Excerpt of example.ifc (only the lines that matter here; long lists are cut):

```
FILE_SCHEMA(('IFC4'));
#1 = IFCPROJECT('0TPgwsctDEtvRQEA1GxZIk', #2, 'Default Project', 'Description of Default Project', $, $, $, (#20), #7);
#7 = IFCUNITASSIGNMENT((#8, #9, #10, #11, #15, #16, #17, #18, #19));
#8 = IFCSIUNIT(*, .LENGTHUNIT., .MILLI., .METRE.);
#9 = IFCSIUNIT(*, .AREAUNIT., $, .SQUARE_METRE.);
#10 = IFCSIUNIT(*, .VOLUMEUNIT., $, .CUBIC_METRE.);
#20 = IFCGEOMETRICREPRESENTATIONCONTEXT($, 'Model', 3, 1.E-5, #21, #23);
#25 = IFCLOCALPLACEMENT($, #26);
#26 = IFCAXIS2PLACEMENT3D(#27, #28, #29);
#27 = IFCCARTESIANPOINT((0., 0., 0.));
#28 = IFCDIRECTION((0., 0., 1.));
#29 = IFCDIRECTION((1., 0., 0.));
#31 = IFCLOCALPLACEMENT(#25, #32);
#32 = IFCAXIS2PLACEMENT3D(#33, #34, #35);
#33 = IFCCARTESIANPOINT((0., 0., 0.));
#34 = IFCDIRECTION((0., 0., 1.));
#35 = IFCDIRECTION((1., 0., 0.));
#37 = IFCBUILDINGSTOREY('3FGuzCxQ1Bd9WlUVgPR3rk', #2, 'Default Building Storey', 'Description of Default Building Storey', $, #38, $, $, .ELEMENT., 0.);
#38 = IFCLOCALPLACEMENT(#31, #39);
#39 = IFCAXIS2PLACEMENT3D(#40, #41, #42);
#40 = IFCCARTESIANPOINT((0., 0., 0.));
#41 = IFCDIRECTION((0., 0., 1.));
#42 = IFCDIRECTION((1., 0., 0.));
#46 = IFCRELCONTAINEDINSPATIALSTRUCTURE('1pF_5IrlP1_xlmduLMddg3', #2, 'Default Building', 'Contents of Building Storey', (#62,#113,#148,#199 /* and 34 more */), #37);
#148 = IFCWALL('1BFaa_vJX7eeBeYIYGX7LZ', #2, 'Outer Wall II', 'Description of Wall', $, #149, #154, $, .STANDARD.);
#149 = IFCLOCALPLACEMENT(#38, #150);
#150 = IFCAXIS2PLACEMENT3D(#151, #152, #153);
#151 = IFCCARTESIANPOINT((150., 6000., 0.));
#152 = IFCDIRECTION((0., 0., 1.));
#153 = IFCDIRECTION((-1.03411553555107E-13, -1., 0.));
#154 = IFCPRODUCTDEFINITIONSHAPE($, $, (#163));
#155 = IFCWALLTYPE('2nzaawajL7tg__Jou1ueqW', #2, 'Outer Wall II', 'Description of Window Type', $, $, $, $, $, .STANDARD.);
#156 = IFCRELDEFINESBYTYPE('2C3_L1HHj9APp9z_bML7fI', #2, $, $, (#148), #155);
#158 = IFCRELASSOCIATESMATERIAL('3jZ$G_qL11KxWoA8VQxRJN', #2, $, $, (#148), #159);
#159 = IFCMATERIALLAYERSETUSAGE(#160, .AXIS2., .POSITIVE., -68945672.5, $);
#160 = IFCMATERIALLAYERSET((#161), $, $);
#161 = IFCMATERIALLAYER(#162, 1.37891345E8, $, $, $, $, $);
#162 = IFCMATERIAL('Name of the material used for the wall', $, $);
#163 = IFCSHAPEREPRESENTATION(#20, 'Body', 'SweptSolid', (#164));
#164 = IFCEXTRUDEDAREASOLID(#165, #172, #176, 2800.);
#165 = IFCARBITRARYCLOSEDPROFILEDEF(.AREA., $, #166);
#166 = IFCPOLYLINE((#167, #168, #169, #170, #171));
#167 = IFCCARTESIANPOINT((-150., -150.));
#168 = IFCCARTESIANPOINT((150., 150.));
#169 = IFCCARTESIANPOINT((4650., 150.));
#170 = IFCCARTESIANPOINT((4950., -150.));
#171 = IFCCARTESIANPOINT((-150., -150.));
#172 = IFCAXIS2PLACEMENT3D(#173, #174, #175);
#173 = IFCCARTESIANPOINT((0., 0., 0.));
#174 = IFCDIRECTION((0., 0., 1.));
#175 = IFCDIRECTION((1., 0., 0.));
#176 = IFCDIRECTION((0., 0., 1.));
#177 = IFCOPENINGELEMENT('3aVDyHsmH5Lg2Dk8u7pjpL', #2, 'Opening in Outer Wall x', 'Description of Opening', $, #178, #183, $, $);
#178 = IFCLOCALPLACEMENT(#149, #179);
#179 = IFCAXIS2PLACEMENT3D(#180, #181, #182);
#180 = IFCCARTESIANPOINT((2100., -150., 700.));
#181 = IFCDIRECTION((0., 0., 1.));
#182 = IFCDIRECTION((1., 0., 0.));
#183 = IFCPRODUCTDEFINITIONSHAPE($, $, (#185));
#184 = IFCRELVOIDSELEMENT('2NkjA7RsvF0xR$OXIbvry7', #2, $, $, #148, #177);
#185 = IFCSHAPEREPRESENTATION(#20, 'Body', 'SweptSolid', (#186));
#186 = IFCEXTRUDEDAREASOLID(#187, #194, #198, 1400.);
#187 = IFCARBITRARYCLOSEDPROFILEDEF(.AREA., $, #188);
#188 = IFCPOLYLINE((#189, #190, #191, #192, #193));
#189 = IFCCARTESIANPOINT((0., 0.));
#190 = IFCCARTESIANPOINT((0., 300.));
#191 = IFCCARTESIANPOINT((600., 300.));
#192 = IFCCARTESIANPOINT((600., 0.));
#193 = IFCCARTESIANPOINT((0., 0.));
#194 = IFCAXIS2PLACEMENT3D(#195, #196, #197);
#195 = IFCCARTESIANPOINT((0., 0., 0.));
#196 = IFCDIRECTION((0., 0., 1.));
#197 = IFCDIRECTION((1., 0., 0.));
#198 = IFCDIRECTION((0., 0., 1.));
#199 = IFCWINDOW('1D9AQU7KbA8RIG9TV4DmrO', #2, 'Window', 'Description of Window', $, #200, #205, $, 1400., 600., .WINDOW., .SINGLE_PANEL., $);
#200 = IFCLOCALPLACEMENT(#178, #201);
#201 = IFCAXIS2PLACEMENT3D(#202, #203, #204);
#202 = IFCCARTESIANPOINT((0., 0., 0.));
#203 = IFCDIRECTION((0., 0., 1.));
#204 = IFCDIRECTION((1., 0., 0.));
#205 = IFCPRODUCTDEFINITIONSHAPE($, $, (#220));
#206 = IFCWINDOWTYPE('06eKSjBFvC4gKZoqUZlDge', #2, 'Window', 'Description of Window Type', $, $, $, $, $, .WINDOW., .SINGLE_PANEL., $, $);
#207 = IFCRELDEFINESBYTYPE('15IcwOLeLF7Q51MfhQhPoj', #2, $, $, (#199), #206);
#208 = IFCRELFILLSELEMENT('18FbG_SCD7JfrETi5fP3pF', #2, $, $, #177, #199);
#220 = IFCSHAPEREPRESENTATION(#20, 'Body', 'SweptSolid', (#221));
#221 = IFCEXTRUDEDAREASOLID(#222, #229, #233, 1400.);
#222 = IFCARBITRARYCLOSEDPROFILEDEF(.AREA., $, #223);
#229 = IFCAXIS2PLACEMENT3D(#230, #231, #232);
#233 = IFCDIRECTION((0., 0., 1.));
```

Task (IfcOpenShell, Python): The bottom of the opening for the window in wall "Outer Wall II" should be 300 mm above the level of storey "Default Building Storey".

```python
import numpy as np
import ifcopenshell
import ifcopenshell.api.geometry
import ifcopenshell.geom
import ifcopenshell.util.element
import ifcopenshell.util.placement
import ifcopenshell.util.shape
import ifcopenshell.util.unit

model = ifcopenshell.open("example.ifc")
unit_scale = ifcopenshell.util.unit.calculate_unit_scale(model)

window = model.by_guid("1D9AQU7KbA8RIG9TV4DmrO")
opening = window.FillsVoids[0].RelatingOpeningElement
storey = ifcopenshell.util.element.get_container(window, ifc_class="IfcBuildingStorey")
level = ifcopenshell.util.placement.get_local_placement(storey.ObjectPlacement)[2, 3]

# The opening's origin need not be at the sill, so measure its lowest point.
shape = ifcopenshell.geom.create_shape(ifcopenshell.geom.settings(), opening)
bottom = ifcopenshell.util.shape.get_shape_bottom_elevation(shape, shape.geometry) / unit_scale
dz = level + 300.0 - bottom

shift = np.array([0.0, 0.0, dz])
# The window is placed relative to its opening, so it follows when the opening moves.
matrix = ifcopenshell.util.placement.get_local_placement(opening.ObjectPlacement)
matrix[:3, 3] += shift
ifcopenshell.api.geometry.edit_object_placement(
    model, product=opening, matrix=matrix, is_si=False, should_transform_children=True
)

print(f"moved by {dz * unit_scale:+.3f} m")

model.write("example_updated.ifc")
```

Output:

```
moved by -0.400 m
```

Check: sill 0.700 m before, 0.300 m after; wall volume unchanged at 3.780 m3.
